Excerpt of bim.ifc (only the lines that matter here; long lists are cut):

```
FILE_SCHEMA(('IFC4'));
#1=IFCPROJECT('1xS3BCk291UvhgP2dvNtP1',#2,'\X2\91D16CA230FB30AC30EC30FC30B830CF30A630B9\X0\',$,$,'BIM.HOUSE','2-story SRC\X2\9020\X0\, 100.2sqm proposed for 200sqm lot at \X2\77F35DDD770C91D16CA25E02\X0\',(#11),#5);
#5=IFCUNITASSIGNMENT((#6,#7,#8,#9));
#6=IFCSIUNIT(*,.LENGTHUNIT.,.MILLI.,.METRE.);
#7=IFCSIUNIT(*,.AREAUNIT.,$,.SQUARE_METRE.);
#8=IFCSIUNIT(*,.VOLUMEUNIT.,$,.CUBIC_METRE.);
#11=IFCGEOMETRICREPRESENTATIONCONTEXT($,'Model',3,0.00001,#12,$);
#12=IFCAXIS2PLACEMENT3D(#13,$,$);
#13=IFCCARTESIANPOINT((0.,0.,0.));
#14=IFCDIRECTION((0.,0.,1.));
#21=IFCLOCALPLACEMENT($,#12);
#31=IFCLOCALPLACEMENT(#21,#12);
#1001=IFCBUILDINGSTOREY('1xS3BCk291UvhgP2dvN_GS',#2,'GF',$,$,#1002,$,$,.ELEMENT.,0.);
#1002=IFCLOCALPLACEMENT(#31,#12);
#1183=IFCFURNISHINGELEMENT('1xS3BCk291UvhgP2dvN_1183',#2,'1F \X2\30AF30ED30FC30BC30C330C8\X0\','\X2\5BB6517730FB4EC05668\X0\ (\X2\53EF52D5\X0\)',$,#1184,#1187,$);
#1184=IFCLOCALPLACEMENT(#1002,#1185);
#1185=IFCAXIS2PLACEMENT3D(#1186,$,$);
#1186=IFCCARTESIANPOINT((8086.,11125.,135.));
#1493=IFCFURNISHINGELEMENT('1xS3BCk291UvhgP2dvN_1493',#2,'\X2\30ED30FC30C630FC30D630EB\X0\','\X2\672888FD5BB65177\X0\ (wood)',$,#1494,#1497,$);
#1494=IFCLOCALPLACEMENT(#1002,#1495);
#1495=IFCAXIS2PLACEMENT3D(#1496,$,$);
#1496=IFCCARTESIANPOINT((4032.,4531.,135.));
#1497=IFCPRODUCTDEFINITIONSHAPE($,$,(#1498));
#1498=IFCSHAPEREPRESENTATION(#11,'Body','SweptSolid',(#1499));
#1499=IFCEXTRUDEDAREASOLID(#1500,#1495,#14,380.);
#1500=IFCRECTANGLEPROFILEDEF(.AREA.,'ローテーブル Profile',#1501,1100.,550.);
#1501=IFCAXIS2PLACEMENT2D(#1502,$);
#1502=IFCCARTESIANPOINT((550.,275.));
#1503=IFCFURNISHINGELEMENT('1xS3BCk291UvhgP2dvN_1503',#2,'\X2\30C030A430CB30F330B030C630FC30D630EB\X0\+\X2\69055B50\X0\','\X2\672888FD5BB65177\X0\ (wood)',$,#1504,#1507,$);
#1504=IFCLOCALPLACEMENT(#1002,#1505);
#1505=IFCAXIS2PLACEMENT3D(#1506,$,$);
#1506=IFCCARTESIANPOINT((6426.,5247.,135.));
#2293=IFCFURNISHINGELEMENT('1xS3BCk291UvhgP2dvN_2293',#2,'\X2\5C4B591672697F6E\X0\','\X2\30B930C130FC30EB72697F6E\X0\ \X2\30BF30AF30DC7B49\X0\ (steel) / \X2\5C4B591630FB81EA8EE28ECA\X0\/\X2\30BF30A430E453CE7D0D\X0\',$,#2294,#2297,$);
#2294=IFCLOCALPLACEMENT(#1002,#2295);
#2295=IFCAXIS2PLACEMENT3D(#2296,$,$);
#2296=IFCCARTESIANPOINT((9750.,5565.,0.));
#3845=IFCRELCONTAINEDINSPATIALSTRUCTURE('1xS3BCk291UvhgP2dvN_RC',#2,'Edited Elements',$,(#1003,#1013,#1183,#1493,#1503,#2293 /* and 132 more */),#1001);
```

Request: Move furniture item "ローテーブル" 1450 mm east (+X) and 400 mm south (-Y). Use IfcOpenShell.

```python
import ifcopenshell
import ifcopenshell.api.geometry
import ifcopenshell.util.placement

model = ifcopenshell.open("bim.ifc")

item = model.by_guid("1xS3BCk291UvhgP2dvN_1493")
matrix = ifcopenshell.util.placement.get_local_placement(item.ObjectPlacement)
matrix[0, 3] += 1450.0
matrix[1, 3] -= 400.0
ifcopenshell.api.geometry.edit_object_placement(model, product=item, matrix=matrix, is_si=False)

print(ifcopenshell.util.placement.get_local_placement(item.ObjectPlacement).round(3) + 0.0)

model.write("bim_updated.ifc")
```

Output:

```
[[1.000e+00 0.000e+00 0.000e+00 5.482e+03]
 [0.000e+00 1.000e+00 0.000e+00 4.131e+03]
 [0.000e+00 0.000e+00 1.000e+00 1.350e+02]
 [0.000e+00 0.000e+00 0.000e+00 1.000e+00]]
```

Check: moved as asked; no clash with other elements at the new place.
